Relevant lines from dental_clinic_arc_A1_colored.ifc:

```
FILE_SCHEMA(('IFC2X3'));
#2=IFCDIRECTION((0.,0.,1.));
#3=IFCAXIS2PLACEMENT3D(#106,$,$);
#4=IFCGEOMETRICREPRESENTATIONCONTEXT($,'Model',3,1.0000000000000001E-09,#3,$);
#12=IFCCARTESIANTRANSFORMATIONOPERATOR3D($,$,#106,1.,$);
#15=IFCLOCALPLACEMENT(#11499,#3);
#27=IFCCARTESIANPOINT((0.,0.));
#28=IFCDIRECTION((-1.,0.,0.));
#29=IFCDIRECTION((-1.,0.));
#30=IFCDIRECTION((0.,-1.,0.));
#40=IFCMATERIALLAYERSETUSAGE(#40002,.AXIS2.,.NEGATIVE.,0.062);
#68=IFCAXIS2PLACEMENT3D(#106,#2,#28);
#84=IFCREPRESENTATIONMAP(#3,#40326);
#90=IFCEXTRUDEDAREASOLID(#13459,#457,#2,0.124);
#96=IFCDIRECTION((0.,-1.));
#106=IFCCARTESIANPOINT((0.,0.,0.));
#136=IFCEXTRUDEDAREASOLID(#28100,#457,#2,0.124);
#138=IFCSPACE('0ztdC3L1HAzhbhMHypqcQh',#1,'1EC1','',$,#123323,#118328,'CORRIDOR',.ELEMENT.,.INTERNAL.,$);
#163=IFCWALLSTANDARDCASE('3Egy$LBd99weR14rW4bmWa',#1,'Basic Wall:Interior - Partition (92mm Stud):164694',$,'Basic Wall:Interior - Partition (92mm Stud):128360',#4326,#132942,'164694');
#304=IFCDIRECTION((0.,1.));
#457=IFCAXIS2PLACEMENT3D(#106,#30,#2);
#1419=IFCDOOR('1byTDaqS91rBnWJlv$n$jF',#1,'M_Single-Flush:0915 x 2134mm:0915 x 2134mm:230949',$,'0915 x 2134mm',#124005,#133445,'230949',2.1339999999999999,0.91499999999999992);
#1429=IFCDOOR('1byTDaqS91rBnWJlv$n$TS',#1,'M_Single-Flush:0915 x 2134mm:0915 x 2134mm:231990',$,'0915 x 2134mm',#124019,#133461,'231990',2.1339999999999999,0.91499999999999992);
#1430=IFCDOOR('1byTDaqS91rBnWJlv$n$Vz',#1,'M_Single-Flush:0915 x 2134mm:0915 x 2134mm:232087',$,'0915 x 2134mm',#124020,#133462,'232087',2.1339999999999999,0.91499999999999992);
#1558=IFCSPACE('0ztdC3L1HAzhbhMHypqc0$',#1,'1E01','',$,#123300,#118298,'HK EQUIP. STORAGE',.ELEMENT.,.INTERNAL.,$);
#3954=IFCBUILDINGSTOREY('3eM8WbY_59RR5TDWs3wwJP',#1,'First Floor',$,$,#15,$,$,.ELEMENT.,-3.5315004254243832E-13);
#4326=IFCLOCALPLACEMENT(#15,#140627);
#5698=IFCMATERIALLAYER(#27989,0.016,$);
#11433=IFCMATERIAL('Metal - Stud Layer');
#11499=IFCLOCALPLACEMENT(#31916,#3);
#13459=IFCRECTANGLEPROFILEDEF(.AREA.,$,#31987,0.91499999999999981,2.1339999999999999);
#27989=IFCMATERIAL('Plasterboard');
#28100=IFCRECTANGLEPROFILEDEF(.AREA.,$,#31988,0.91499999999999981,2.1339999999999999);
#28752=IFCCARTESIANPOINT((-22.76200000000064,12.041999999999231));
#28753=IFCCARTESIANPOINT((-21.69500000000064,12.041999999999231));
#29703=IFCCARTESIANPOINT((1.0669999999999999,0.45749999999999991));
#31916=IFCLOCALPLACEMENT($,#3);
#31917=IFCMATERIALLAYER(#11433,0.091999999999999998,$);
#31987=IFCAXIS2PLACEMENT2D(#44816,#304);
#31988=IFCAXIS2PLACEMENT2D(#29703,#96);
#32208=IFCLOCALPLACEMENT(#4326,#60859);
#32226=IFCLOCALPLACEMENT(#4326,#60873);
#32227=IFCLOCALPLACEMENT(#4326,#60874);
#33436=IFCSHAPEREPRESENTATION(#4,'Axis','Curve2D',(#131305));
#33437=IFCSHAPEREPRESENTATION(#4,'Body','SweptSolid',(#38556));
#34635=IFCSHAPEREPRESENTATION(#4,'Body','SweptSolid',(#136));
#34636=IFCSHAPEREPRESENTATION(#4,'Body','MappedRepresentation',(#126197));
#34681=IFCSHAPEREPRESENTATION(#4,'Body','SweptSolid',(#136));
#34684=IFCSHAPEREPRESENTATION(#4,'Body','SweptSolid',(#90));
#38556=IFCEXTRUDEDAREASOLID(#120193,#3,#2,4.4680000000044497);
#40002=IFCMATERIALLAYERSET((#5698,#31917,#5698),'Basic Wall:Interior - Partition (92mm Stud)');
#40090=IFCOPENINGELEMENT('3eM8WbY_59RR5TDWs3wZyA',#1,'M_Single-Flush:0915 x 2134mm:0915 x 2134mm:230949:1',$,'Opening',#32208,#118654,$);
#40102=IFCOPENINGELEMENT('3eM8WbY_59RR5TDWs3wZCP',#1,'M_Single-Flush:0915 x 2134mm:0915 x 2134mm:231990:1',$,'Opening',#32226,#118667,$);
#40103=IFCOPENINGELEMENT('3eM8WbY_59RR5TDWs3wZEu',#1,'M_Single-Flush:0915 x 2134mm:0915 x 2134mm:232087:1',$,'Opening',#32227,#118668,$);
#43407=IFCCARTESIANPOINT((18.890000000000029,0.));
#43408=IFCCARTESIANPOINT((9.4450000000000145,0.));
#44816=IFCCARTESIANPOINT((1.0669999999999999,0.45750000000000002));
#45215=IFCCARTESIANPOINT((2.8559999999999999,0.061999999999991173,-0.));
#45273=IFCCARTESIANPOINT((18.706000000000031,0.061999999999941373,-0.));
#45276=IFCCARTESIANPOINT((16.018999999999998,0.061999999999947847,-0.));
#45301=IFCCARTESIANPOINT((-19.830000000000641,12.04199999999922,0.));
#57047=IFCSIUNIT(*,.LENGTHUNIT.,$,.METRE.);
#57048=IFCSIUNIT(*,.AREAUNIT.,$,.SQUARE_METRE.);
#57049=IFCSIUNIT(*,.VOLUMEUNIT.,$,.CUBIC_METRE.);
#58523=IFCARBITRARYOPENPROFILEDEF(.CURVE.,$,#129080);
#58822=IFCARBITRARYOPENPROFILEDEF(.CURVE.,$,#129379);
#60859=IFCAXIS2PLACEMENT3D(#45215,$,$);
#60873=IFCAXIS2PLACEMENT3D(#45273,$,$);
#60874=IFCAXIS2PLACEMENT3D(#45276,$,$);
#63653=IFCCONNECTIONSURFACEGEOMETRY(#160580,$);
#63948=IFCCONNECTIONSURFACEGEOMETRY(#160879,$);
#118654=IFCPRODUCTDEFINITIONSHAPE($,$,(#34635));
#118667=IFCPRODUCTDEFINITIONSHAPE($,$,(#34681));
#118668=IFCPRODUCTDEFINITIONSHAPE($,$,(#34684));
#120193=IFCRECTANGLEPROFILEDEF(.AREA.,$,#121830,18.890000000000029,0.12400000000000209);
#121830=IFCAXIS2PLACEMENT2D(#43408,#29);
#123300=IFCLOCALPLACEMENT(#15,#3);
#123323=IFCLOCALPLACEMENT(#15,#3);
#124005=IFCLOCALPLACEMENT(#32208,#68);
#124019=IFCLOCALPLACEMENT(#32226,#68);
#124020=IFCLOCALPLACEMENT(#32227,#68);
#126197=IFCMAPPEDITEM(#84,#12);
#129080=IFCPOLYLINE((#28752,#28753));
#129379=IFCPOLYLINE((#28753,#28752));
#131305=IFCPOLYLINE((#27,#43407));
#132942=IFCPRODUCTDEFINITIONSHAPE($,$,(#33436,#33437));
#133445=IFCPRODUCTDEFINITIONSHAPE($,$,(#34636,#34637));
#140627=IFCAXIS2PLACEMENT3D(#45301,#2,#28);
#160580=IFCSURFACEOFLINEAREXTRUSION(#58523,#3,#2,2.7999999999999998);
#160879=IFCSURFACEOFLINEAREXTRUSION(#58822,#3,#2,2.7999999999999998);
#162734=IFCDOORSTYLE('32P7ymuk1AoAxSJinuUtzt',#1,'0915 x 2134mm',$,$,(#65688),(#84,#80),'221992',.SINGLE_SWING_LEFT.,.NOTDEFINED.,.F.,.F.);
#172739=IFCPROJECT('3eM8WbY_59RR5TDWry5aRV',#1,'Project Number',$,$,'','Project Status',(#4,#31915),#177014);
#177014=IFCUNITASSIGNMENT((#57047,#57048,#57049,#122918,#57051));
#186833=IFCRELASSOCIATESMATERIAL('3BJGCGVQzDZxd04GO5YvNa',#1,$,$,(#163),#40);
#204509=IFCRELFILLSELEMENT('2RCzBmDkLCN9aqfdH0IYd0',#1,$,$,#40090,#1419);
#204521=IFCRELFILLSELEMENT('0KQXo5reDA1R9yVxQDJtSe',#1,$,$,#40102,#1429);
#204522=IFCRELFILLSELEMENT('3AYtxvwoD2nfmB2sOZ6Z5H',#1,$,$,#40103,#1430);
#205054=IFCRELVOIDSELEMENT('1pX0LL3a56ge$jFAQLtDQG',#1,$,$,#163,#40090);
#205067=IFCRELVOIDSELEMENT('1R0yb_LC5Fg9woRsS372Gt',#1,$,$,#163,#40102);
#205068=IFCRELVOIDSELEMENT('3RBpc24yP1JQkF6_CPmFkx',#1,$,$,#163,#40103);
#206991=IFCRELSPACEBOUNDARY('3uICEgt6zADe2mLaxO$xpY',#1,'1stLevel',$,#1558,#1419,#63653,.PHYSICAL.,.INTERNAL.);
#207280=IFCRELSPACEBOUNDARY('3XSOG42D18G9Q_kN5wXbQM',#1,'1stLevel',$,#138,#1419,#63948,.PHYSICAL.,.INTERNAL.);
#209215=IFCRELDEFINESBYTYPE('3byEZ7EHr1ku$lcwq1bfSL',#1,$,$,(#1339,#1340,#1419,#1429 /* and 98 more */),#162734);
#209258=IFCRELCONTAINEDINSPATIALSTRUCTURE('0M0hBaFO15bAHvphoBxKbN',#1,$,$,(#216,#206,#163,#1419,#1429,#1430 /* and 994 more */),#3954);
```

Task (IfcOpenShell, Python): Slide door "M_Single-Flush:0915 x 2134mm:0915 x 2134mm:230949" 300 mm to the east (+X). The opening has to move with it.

```python
import numpy as np
import ifcopenshell
import ifcopenshell.api.geometry
import ifcopenshell.util.placement
import ifcopenshell.util.unit

model = ifcopenshell.open("dental_clinic_arc_A1_colored.ifc")
unit_scale = ifcopenshell.util.unit.calculate_unit_scale(model)

door = model.by_guid("1byTDaqS91rBnWJlv$n$jF")
opening = door.FillsVoids[0].RelatingOpeningElement
wall = opening.VoidsElements[0].RelatingBuildingElement

wall_matrix = ifcopenshell.util.placement.get_local_placement(wall.ObjectPlacement)
shift = wall_matrix[:3, 0] * -0.3 / unit_scale
before = ifcopenshell.util.placement.get_local_placement(door.ObjectPlacement)[:3, 3].copy()

# The door is placed relative to its opening, so it follows when the opening moves.
matrix = ifcopenshell.util.placement.get_local_placement(opening.ObjectPlacement)
matrix[:3, 3] += shift
ifcopenshell.api.geometry.edit_object_placement(
    model, product=opening, matrix=matrix, is_si=False, should_transform_children=True
)

# Space boundary surfaces are stored in each space's coordinates; move them too.
for rel in door.ProvidesBoundaries:
    if not rel.ConnectionGeometry:
        continue
    surface = rel.ConnectionGeometry.SurfaceOnRelatingElement
    space_matrix = ifcopenshell.util.placement.get_local_placement(rel.RelatingSpace.ObjectPlacement)
    point = np.array(surface.Position.Location.Coordinates) + space_matrix[:3, :3].T @ shift
    surface.Position = model.createIfcAxis2Placement3D(
        model.createIfcCartesianPoint(point.tolist()), surface.Position.Axis, surface.Position.RefDirection
    )

after = ifcopenshell.util.placement.get_local_placement(door.ObjectPlacement)[:3, 3]
print("door moved by", (after - before).round(3) + 0.0)

model.write("dental_clinic_arc_A1_colored_v2.ifc")
```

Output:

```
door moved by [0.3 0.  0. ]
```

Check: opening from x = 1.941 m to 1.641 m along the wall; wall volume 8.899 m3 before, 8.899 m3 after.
